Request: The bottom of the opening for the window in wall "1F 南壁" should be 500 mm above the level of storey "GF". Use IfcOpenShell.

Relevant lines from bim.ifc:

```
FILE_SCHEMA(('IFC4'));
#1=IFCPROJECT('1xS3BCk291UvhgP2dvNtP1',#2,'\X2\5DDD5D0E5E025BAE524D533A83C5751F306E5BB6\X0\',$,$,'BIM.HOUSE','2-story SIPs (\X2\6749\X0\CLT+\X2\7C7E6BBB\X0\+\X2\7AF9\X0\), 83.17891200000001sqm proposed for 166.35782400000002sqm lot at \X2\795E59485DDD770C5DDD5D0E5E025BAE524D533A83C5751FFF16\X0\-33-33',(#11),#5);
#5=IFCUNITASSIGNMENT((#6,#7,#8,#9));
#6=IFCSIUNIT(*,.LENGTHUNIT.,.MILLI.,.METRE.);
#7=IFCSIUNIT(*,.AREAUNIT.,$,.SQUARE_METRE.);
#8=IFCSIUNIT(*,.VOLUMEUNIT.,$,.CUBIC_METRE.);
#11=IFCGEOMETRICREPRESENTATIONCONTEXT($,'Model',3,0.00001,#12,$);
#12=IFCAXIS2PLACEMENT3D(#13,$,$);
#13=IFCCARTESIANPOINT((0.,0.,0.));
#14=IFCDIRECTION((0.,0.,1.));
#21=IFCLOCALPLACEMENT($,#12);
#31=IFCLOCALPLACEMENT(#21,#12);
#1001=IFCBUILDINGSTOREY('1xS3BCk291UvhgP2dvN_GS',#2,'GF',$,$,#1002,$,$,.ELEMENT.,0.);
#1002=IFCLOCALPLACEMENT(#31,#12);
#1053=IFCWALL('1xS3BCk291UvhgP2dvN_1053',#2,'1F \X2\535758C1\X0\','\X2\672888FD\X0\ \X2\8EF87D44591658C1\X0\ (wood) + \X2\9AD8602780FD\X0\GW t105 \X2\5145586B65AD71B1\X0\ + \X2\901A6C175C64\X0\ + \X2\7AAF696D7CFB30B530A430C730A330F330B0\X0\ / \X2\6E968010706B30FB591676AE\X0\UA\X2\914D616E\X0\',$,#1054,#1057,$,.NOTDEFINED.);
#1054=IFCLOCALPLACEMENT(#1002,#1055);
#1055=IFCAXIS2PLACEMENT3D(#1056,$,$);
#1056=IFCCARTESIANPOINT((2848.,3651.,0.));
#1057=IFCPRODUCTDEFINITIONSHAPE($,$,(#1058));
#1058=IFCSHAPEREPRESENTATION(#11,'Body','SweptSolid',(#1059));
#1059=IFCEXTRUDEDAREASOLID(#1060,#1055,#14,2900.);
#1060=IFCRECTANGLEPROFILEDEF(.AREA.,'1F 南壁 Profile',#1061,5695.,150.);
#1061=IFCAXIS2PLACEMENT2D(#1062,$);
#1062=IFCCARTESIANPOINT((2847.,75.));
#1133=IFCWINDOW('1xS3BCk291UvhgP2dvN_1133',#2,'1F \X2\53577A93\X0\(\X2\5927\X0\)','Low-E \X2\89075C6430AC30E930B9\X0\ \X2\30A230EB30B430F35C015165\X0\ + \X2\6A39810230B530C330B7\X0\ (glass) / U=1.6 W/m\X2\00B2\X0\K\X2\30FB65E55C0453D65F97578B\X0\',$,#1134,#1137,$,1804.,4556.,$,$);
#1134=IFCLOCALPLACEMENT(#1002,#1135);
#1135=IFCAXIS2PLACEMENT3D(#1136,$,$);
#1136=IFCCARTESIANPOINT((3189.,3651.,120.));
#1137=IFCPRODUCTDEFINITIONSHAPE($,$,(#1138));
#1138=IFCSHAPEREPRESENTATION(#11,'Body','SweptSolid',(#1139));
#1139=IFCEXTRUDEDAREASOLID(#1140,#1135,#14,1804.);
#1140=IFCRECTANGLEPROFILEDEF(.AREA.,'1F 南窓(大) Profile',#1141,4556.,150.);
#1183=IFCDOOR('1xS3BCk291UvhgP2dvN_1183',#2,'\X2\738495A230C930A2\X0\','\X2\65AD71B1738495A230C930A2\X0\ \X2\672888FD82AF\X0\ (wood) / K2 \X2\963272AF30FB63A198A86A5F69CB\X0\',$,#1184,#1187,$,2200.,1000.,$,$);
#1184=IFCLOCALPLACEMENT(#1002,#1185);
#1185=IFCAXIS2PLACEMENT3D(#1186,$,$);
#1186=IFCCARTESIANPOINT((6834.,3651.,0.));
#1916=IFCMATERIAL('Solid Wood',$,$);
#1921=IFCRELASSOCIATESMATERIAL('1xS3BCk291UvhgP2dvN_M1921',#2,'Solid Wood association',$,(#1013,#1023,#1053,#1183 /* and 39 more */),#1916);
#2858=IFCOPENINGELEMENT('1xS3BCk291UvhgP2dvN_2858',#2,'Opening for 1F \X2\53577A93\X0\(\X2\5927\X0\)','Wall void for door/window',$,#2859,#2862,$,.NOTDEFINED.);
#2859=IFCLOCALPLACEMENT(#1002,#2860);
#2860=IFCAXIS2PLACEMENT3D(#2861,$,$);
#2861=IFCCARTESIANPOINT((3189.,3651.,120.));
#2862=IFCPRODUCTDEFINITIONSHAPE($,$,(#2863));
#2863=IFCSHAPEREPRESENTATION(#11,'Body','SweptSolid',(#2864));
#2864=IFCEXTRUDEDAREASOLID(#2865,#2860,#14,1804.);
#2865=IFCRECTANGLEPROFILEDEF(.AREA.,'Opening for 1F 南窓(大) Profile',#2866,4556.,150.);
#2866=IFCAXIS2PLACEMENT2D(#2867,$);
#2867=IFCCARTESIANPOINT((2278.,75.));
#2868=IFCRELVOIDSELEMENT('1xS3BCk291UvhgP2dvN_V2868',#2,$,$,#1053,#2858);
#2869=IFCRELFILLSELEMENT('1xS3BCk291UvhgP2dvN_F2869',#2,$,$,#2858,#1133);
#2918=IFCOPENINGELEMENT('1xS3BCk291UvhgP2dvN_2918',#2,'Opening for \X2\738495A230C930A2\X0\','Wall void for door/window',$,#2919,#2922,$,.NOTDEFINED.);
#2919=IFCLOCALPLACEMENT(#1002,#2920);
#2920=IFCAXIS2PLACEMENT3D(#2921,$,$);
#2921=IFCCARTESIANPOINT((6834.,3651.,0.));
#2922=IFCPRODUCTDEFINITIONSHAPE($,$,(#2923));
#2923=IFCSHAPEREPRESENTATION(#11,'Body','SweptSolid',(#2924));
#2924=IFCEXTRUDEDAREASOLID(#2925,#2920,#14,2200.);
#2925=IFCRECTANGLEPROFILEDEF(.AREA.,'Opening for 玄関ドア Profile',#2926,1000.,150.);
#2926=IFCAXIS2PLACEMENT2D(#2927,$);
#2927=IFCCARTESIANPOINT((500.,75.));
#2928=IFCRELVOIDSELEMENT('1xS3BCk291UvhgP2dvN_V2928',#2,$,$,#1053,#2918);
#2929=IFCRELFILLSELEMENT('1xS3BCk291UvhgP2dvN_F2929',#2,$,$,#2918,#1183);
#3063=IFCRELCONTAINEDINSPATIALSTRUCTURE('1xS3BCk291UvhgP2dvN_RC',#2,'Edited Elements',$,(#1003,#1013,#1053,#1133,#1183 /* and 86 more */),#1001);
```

```python
import numpy as np
import ifcopenshell
import ifcopenshell.api.geometry
import ifcopenshell.geom
import ifcopenshell.util.element
import ifcopenshell.util.placement
import ifcopenshell.util.shape
import ifcopenshell.util.unit

model = ifcopenshell.open("bim.ifc")
unit_scale = ifcopenshell.util.unit.calculate_unit_scale(model)

window = model.by_id(1133)
opening = window.FillsVoids[0].RelatingOpeningElement
storey = ifcopenshell.util.element.get_container(window, ifc_class="IfcBuildingStorey")
level = ifcopenshell.util.placement.get_local_placement(storey.ObjectPlacement)[2, 3]

# The opening's origin need not be at the sill, so measure its lowest point.
shape = ifcopenshell.geom.create_shape(ifcopenshell.geom.settings(), opening)
bottom = ifcopenshell.util.shape.get_shape_bottom_elevation(shape, shape.geometry) / unit_scale
dz = level + 0.5 / unit_scale - bottom

shift = np.array([0.0, 0.0, dz])
# The window is not placed relative to its opening, so move both.
for product in (opening, window):
    matrix = ifcopenshell.util.placement.get_local_placement(product.ObjectPlacement)
    matrix[:3, 3] += shift
    ifcopenshell.api.geometry.edit_object_placement(model, product=product, matrix=matrix, is_si=False)

print(f"moved by {dz * unit_scale:+.3f} m")

model.write("bim_edited.ifc")
```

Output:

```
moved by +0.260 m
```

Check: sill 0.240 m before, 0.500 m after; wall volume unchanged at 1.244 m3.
